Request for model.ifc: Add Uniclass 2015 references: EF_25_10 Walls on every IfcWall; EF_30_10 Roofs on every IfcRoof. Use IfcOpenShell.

First a look at what the model holds.

```python
import ifcopenshell

model = ifcopenshell.open("model.ifc")
print(model.schema)
print("classifications:", [c.Name for c in model.by_type("IfcClassification")])
for ifc_class in ("IfcDoor", "IfcRoof", "IfcStair", "IfcWall", "IfcWindow"):
    print(ifc_class, len(model.by_type(ifc_class)))
```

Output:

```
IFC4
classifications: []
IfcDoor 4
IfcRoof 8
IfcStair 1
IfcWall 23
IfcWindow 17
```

```python
import ifcopenshell
import ifcopenshell.api.classification

model = ifcopenshell.open("model.ifc")

system = ifcopenshell.api.classification.add_classification(model, classification="Uniclass 2015")

codes = {
    "IfcWall": ("EF_25_10", "Walls"),
    "IfcRoof": ("EF_30_10", "Roofs"),
}
for ifc_class, (code, name) in codes.items():
    products = model.by_type(ifc_class)
    ifcopenshell.api.classification.add_reference(
        model, products=products, classification=system, identification=code, name=name
    )
    print(code, len(products))

model.write("model_v2.ifc")
```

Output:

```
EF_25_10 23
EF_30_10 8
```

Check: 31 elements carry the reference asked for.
